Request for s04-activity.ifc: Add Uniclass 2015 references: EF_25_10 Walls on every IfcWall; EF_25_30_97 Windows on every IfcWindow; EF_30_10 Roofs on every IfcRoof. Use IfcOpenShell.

First a look at what the model holds.

```python
import ifcopenshell

model = ifcopenshell.open("s04-activity.ifc")
print(model.schema)
print("classifications:", [c.Name for c in model.by_type("IfcClassification")])
for ifc_class in ("IfcDoor", "IfcRoof", "IfcStair", "IfcWall", "IfcWindow"):
    print(ifc_class, len(model.by_type(ifc_class)))
```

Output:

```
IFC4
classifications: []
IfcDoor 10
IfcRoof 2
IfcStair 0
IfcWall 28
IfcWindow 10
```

```python
import ifcopenshell
import ifcopenshell.api.classification

model = ifcopenshell.open("s04-activity.ifc")

system = ifcopenshell.api.classification.add_classification(model, classification="Uniclass 2015")

codes = {
    "IfcWall": ("EF_25_10", "Walls"),
    "IfcWindow": ("EF_25_30_97", "Windows"),
    "IfcRoof": ("EF_30_10", "Roofs"),
}
for ifc_class, (code, name) in codes.items():
    products = model.by_type(ifc_class)
    ifcopenshell.api.classification.add_reference(
        model, products=products, classification=system, identification=code, name=name
    )
    print(code, len(products))

model.write("s04-activity_edited.ifc")
```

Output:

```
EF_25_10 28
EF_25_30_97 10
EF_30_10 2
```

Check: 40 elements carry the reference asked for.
